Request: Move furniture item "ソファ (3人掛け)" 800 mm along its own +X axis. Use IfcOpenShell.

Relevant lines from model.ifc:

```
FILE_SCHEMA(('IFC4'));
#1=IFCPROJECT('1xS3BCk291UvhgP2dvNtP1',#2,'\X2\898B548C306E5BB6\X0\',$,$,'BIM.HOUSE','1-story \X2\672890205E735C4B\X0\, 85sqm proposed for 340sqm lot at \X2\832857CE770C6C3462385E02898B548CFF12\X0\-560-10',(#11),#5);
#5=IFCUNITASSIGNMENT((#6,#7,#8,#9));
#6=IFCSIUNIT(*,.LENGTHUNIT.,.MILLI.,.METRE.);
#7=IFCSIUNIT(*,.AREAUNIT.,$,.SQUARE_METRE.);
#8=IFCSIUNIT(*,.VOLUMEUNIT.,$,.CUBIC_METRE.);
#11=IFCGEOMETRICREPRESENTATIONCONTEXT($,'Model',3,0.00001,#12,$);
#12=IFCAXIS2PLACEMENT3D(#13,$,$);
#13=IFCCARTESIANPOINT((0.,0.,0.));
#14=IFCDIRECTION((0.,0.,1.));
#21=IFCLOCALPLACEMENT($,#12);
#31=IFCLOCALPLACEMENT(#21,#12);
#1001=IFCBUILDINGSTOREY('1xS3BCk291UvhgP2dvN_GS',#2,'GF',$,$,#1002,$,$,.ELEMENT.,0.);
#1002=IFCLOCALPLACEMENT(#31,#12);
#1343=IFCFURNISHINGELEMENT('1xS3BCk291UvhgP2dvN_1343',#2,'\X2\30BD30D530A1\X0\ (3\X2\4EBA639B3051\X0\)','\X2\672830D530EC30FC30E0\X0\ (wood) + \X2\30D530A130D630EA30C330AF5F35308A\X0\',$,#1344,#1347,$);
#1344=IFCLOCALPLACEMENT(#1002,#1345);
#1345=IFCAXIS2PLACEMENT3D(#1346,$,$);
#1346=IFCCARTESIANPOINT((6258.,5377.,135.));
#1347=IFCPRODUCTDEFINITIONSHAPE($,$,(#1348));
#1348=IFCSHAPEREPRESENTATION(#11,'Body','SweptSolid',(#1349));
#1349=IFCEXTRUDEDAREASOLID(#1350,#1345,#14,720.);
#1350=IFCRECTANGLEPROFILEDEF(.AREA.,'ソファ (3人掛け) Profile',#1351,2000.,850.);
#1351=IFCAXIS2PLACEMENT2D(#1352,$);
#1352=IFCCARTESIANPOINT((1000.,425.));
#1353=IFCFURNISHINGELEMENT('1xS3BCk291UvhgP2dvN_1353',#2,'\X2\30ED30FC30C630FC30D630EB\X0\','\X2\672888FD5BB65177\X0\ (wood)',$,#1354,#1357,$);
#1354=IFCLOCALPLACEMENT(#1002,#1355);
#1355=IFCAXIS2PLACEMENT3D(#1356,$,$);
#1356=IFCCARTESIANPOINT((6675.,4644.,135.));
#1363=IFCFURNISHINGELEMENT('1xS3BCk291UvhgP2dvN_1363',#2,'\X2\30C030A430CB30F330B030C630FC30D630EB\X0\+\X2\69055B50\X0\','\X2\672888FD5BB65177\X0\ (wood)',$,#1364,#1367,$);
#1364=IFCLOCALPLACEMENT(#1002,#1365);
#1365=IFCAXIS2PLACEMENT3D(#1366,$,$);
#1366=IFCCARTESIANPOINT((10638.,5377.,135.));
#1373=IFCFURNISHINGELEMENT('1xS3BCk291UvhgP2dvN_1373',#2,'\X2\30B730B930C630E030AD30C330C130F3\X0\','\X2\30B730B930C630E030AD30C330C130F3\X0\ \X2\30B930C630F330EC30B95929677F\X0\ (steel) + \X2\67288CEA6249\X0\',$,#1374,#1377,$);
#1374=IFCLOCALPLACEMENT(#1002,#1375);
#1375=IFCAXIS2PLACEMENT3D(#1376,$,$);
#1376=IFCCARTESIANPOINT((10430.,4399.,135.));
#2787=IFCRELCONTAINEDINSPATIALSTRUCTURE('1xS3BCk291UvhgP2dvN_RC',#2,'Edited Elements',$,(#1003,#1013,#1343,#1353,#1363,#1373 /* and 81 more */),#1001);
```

```python
import ifcopenshell
import ifcopenshell.api.geometry
import ifcopenshell.util.placement

model = ifcopenshell.open("model.ifc")

item = model.by_guid("1xS3BCk291UvhgP2dvN_1343")
matrix = ifcopenshell.util.placement.get_local_placement(item.ObjectPlacement)
matrix[:3, 3] += matrix[:3, 0] * 800.0
ifcopenshell.api.geometry.edit_object_placement(model, product=item, matrix=matrix, is_si=False)

print(ifcopenshell.util.placement.get_local_placement(item.ObjectPlacement).round(3) + 0.0)

model.write("model_rev.ifc")
```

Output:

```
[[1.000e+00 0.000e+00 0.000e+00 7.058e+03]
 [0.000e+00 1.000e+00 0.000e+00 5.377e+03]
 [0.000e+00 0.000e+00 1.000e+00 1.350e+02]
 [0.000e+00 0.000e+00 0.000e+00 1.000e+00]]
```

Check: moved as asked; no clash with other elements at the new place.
